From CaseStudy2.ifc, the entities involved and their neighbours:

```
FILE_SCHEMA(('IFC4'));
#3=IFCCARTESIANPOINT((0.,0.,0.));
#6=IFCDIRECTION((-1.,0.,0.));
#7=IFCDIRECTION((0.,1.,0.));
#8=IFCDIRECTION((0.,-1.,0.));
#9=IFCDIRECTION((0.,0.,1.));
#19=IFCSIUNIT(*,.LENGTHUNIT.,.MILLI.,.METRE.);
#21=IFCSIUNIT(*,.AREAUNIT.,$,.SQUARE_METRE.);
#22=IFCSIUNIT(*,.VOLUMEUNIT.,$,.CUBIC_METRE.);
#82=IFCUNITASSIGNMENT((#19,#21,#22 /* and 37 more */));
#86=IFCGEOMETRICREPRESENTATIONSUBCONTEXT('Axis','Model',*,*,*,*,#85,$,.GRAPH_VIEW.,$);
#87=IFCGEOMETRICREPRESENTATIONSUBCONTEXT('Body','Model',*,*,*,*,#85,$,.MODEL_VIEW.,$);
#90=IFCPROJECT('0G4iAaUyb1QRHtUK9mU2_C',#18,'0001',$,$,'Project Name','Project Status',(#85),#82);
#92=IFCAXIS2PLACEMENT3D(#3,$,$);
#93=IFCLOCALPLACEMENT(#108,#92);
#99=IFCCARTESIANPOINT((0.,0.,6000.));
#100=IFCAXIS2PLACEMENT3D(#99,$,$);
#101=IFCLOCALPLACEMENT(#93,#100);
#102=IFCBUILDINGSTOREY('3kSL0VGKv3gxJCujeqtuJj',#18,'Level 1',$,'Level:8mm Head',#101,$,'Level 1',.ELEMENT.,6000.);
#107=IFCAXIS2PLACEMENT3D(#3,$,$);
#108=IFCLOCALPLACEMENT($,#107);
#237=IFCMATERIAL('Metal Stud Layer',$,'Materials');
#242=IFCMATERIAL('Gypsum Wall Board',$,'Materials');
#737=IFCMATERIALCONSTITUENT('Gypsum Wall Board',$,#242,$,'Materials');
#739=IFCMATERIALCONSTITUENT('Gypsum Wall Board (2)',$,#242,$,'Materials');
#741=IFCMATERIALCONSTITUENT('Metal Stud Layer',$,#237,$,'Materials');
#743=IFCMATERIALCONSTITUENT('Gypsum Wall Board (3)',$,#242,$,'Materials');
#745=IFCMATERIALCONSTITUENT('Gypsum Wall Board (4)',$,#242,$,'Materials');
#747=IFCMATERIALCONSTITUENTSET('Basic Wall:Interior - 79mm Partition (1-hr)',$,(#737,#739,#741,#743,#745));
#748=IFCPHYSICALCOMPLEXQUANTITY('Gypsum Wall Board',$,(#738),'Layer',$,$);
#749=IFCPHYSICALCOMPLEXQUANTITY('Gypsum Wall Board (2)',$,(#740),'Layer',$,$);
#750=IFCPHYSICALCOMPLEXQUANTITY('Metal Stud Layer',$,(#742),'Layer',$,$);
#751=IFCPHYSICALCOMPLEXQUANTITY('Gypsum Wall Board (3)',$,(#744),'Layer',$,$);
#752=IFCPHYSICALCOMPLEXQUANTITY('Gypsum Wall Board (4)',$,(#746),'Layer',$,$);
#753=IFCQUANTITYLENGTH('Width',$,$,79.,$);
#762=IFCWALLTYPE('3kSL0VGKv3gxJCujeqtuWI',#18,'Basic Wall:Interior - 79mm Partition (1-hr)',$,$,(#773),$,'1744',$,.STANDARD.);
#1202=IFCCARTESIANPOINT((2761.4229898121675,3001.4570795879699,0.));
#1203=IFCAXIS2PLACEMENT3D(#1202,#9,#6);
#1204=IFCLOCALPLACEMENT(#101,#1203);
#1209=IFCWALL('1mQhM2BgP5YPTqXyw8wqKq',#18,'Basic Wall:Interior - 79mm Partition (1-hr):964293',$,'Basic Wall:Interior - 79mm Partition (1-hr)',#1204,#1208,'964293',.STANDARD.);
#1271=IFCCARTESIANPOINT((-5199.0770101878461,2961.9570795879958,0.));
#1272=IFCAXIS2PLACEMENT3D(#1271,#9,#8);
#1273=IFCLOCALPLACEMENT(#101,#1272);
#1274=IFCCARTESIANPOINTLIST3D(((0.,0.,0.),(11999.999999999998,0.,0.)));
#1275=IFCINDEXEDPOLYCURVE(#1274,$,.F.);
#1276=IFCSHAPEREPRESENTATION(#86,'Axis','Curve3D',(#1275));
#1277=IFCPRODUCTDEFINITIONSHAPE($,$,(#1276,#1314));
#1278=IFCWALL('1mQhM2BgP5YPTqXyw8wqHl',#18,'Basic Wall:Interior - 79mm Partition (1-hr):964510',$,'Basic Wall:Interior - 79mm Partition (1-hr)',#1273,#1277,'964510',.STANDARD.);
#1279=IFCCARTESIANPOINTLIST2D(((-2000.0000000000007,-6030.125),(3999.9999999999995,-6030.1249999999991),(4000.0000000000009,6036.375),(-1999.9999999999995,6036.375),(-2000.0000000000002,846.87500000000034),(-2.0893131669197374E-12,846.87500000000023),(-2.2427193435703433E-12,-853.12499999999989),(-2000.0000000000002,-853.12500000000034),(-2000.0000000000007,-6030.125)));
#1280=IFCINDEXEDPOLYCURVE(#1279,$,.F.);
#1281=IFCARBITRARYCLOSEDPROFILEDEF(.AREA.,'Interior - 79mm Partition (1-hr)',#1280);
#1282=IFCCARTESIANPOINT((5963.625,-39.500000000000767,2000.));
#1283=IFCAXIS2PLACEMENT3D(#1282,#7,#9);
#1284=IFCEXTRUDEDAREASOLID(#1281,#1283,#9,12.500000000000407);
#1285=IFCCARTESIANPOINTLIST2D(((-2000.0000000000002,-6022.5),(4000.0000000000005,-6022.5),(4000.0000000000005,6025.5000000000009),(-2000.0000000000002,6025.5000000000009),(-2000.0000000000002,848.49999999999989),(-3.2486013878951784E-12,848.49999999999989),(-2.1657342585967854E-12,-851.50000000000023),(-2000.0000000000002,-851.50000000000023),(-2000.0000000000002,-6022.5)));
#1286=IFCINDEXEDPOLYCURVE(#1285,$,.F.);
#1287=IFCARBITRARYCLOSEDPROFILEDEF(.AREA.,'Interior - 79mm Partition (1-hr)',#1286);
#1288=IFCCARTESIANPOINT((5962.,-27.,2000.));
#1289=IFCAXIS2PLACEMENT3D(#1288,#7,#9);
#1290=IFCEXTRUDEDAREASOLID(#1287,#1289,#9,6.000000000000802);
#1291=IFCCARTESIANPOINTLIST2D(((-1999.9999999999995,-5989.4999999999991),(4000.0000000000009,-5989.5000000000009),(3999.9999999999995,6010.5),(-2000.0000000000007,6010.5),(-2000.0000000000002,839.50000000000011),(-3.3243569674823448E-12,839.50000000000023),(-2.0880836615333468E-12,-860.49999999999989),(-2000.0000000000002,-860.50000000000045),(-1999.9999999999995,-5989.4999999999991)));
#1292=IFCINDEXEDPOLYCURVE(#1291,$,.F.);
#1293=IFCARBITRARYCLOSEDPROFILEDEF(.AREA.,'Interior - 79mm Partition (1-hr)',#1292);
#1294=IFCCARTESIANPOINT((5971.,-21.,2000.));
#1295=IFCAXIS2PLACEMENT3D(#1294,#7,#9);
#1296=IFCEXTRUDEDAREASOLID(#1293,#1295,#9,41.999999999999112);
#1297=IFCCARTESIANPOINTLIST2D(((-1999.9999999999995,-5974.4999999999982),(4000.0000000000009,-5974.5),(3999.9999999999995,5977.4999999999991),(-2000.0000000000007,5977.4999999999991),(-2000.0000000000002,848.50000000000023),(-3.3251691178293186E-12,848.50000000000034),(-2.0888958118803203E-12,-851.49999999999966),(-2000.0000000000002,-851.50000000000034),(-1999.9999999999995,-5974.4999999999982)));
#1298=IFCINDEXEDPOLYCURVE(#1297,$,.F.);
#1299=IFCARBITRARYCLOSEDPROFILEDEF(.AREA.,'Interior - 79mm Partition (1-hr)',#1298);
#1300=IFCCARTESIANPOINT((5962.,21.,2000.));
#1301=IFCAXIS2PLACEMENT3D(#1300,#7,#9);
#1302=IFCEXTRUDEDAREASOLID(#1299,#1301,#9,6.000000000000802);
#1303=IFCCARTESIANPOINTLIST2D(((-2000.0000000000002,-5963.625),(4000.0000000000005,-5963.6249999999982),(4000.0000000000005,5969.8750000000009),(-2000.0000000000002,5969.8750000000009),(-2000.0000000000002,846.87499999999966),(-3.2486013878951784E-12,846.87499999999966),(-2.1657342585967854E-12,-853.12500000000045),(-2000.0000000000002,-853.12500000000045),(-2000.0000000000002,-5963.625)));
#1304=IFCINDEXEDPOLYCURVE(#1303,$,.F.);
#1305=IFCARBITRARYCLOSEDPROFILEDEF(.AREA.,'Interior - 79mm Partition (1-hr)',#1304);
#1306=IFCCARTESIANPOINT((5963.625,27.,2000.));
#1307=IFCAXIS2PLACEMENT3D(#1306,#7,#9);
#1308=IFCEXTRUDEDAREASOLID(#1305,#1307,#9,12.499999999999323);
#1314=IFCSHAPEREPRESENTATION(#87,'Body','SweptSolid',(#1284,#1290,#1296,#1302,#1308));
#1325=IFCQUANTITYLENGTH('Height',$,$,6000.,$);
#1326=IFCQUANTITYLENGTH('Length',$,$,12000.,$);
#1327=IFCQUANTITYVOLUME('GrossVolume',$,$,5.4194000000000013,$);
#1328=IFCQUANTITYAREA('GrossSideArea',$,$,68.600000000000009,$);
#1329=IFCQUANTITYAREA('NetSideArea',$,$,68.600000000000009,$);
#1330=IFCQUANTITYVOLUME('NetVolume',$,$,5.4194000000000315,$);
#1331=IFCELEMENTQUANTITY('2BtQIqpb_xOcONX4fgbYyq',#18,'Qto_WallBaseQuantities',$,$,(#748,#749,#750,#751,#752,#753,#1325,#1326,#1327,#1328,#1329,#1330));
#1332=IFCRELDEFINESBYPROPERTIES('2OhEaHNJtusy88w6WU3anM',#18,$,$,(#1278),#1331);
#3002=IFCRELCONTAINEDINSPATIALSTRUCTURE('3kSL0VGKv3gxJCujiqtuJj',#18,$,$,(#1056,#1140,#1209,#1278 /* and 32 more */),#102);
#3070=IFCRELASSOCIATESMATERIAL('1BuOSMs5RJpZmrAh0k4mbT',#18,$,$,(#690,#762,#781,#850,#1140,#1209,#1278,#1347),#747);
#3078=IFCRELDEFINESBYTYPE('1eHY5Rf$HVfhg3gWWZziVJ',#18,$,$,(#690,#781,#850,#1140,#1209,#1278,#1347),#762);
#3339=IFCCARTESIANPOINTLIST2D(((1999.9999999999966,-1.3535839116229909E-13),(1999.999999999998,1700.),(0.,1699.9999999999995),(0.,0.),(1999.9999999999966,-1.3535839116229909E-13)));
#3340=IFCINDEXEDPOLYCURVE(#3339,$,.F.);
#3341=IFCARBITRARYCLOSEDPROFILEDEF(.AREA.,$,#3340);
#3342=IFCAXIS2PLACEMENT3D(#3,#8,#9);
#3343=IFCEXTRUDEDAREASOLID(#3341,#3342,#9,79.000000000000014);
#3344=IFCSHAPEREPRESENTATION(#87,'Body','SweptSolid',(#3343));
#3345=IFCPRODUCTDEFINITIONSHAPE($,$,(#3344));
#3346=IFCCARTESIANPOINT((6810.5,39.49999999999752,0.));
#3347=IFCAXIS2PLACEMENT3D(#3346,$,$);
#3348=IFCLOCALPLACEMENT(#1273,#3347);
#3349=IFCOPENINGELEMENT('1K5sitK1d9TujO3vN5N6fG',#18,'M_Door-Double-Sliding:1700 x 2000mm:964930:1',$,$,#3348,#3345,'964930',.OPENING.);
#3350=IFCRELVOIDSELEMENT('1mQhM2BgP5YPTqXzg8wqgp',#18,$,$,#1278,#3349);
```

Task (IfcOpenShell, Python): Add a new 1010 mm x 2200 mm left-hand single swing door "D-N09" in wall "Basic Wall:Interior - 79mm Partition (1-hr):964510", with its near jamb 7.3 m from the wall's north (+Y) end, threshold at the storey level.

```python
import numpy as np
import ifcopenshell
import ifcopenshell.api.feature
import ifcopenshell.api.geometry
import ifcopenshell.api.pset
import ifcopenshell.api.root
import ifcopenshell.api.spatial
import ifcopenshell.geom
import ifcopenshell.util.element
import ifcopenshell.util.placement
import ifcopenshell.util.representation
import ifcopenshell.util.shape
import ifcopenshell.util.unit

model = ifcopenshell.open("CaseStudy2.ifc")
unit_scale = ifcopenshell.util.unit.calculate_unit_scale(model)
area_scale = ifcopenshell.util.unit.calculate_unit_scale(model, "AREAUNIT")
volume_scale = ifcopenshell.util.unit.calculate_unit_scale(model, "VOLUMEUNIT")
settings = ifcopenshell.geom.settings()


def volume(element):
    """Net volume in cubic metres, openings subtracted."""
    shape = ifcopenshell.geom.create_shape(settings, element)
    return ifcopenshell.util.shape.get_volume(shape.geometry)


wall = model.by_guid("1mQhM2BgP5YPTqXyw8wqHl")
storey = ifcopenshell.util.element.get_container(wall, ifc_class="IfcBuildingStorey")
context = ifcopenshell.util.representation.get_context(model, "Model", "Body", "MODEL_VIEW")
before = volume(wall)

width, height, from_end, sill = 1.01, 2.2, 7.3, 0.0  # metres

# The wall runs along its own X axis, and the end named is its -X end.
wall_shape = ifcopenshell.geom.create_shape(settings, wall)
x, y, z = ifcopenshell.util.shape.get_vertices(wall_shape.geometry).T
start = x.min() + from_end
face, thickness = float(y.min()), float(y.max() - y.min())
wall_matrix = ifcopenshell.util.placement.get_local_placement(wall.ObjectPlacement)
level = ifcopenshell.util.placement.get_local_placement(storey.ObjectPlacement)[2, 3]


def in_wall(x, y):
    """Placement at x, y metres in the wall's axes, at sill height."""
    matrix = wall_matrix.copy()
    matrix[:, 3] = wall_matrix @ np.array([x / unit_scale, y / unit_scale, 0.0, 1.0])
    matrix[2, 3] = level + sill / unit_scale
    return matrix


# Opening: a box that overshoots both wall faces by 50 mm.
opening = ifcopenshell.api.root.create_entity(model, ifc_class="IfcOpeningElement", predefined_type="OPENING")
box = ifcopenshell.api.geometry.add_wall_representation(
    model, context=context, length=width, height=height, thickness=thickness + 0.1
)
ifcopenshell.api.geometry.assign_representation(model, product=opening, representation=box)
ifcopenshell.api.geometry.edit_object_placement(model, product=opening, matrix=in_wall(start, face - 0.05), is_si=False)
ifcopenshell.api.feature.add_feature(model, feature=opening, element=wall)

door = ifcopenshell.api.root.create_entity(model, ifc_class="IfcDoor", name="D-N09", predefined_type="DOOR")
door.OverallWidth, door.OverallHeight = width / unit_scale, height / unit_scale
door.OperationType = "SINGLE_SWING_LEFT"
body = ifcopenshell.api.geometry.add_door_representation(
    model,
    context=context,
    overall_width=door.OverallWidth,
    overall_height=door.OverallHeight,
    operation_type="SINGLE_SWING_LEFT",
    lining_properties={"LiningDepth": thickness / unit_scale, "ThresholdDepth": thickness / unit_scale},
)
ifcopenshell.api.geometry.assign_representation(model, product=door, representation=body)
ifcopenshell.api.spatial.assign_container(model, products=[door], relating_structure=storey)
ifcopenshell.api.feature.add_filling(model, opening=opening, element=door)

# The lining spans the wall, so the door starts at the wall face.
ifcopenshell.api.geometry.edit_object_placement(model, product=door, matrix=in_wall(start, face), is_si=False)

after = volume(wall)

# Update the wall's stored quantities.
qto = model.by_id(ifcopenshell.util.element.get_pset(wall, "Qto_WallBaseQuantities", should_inherit=False)["id"])
ifcopenshell.api.pset.edit_qto(model, qto=qto, properties={
    "NetSideArea": after / thickness / area_scale,
    "NetVolume": after / volume_scale,
})

print(f"wall volume {before:.3f} -> {after:.3f} m3")

model.write("CaseStudy2-out.ifc")
```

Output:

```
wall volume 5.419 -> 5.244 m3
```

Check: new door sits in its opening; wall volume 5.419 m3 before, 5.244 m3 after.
